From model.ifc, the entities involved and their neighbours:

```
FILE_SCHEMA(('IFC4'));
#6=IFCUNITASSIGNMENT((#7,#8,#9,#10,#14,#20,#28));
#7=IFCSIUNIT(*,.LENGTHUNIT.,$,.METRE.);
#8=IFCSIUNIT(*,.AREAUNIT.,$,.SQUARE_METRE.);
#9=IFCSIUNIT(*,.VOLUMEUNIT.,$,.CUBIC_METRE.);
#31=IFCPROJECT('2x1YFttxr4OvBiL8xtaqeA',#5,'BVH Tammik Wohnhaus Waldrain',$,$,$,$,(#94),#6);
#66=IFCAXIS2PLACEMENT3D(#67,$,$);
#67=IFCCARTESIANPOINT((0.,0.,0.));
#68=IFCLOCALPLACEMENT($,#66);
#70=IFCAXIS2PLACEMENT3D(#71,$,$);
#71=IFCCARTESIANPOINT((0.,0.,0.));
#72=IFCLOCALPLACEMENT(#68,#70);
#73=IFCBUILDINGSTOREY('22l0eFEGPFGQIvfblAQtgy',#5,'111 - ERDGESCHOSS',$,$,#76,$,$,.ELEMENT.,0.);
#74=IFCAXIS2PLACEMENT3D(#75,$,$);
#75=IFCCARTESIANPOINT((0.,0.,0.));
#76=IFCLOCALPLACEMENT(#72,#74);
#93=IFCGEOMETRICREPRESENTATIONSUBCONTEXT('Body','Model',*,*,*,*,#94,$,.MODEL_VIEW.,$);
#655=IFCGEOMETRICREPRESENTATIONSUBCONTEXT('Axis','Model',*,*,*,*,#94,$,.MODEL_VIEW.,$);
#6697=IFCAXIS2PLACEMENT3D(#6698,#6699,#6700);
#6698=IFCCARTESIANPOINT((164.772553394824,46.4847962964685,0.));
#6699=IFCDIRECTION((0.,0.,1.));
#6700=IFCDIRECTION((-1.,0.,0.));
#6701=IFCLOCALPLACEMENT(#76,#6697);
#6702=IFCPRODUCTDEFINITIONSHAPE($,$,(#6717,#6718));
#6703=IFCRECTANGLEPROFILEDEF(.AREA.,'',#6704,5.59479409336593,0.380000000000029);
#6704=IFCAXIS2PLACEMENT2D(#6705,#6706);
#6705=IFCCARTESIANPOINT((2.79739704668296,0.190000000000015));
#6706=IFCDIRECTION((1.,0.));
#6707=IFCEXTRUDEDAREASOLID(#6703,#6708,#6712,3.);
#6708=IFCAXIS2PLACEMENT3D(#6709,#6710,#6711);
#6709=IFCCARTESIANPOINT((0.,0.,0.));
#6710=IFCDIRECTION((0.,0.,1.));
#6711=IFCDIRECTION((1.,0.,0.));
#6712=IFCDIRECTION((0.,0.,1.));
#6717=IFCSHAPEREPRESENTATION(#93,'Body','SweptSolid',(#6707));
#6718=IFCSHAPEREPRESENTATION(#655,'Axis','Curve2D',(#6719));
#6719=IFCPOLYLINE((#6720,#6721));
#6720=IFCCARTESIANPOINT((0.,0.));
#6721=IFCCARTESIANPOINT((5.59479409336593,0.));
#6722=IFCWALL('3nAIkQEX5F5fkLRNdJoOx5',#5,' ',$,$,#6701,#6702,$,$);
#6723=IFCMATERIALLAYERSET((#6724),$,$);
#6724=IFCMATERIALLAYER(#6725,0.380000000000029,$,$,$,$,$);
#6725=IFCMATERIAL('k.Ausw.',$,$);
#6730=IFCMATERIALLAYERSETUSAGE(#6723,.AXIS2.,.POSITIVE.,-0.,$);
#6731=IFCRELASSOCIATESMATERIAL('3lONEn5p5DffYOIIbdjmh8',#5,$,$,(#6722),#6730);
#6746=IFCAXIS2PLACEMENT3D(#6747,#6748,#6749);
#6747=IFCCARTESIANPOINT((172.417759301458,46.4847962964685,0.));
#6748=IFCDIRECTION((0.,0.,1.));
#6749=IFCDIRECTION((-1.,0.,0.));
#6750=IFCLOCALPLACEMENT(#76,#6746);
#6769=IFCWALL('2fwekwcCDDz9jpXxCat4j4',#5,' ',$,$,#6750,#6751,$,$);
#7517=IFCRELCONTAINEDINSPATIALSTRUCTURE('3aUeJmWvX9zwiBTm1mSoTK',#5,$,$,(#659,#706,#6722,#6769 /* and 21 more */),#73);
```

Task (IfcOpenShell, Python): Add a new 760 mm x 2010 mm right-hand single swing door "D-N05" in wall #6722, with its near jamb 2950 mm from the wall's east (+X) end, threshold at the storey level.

```python
import numpy as np
import ifcopenshell
import ifcopenshell.api.feature
import ifcopenshell.api.geometry
import ifcopenshell.api.root
import ifcopenshell.api.spatial
import ifcopenshell.geom
import ifcopenshell.util.element
import ifcopenshell.util.placement
import ifcopenshell.util.representation
import ifcopenshell.util.shape
import ifcopenshell.util.unit

model = ifcopenshell.open("model.ifc")
unit_scale = ifcopenshell.util.unit.calculate_unit_scale(model)
settings = ifcopenshell.geom.settings()


def volume(element):
    """Net volume in cubic metres, openings subtracted."""
    shape = ifcopenshell.geom.create_shape(settings, element)
    return ifcopenshell.util.shape.get_volume(shape.geometry)


wall = model.by_guid("3nAIkQEX5F5fkLRNdJoOx5")
storey = ifcopenshell.util.element.get_container(wall, ifc_class="IfcBuildingStorey")
context = ifcopenshell.util.representation.get_context(model, "Model", "Body", "MODEL_VIEW")
before = volume(wall)

width, height, from_end, sill = 0.76, 2.01, 2.95, 0.0  # metres

# The wall runs along its own X axis, and the end named is its -X end.
wall_shape = ifcopenshell.geom.create_shape(settings, wall)
x, y, z = ifcopenshell.util.shape.get_vertices(wall_shape.geometry).T
start = x.min() + from_end
face, thickness = float(y.min()), float(y.max() - y.min())
wall_matrix = ifcopenshell.util.placement.get_local_placement(wall.ObjectPlacement)
level = ifcopenshell.util.placement.get_local_placement(storey.ObjectPlacement)[2, 3]


def in_wall(x, y):
    """Placement at x, y metres in the wall's axes, at sill height."""
    matrix = wall_matrix.copy()
    matrix[:, 3] = wall_matrix @ np.array([x / unit_scale, y / unit_scale, 0.0, 1.0])
    matrix[2, 3] = level + sill / unit_scale
    return matrix


# Opening: a box that overshoots both wall faces by 50 mm.
opening = ifcopenshell.api.root.create_entity(model, ifc_class="IfcOpeningElement", predefined_type="OPENING")
box = ifcopenshell.api.geometry.add_wall_representation(
    model, context=context, length=width, height=height, thickness=thickness + 0.1
)
ifcopenshell.api.geometry.assign_representation(model, product=opening, representation=box)
ifcopenshell.api.geometry.edit_object_placement(model, product=opening, matrix=in_wall(start, face - 0.05), is_si=False)
ifcopenshell.api.feature.add_feature(model, feature=opening, element=wall)

door = ifcopenshell.api.root.create_entity(model, ifc_class="IfcDoor", name="D-N05", predefined_type="DOOR")
door.OverallWidth, door.OverallHeight = width / unit_scale, height / unit_scale
door.OperationType = "SINGLE_SWING_RIGHT"
body = ifcopenshell.api.geometry.add_door_representation(
    model,
    context=context,
    overall_width=door.OverallWidth,
    overall_height=door.OverallHeight,
    operation_type="SINGLE_SWING_RIGHT",
    lining_properties={"LiningDepth": thickness / unit_scale, "ThresholdDepth": thickness / unit_scale},
)
ifcopenshell.api.geometry.assign_representation(model, product=door, representation=body)
ifcopenshell.api.spatial.assign_container(model, products=[door], relating_structure=storey)
ifcopenshell.api.feature.add_filling(model, opening=opening, element=door)

# The lining spans the wall, so the door starts at the wall face.
ifcopenshell.api.geometry.edit_object_placement(model, product=door, matrix=in_wall(start, face), is_si=False)

after = volume(wall)

print(f"wall volume {before:.3f} -> {after:.3f} m3")

model.write("model_rev.ifc")
```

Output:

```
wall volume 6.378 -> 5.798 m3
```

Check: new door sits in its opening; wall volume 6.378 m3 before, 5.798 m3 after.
